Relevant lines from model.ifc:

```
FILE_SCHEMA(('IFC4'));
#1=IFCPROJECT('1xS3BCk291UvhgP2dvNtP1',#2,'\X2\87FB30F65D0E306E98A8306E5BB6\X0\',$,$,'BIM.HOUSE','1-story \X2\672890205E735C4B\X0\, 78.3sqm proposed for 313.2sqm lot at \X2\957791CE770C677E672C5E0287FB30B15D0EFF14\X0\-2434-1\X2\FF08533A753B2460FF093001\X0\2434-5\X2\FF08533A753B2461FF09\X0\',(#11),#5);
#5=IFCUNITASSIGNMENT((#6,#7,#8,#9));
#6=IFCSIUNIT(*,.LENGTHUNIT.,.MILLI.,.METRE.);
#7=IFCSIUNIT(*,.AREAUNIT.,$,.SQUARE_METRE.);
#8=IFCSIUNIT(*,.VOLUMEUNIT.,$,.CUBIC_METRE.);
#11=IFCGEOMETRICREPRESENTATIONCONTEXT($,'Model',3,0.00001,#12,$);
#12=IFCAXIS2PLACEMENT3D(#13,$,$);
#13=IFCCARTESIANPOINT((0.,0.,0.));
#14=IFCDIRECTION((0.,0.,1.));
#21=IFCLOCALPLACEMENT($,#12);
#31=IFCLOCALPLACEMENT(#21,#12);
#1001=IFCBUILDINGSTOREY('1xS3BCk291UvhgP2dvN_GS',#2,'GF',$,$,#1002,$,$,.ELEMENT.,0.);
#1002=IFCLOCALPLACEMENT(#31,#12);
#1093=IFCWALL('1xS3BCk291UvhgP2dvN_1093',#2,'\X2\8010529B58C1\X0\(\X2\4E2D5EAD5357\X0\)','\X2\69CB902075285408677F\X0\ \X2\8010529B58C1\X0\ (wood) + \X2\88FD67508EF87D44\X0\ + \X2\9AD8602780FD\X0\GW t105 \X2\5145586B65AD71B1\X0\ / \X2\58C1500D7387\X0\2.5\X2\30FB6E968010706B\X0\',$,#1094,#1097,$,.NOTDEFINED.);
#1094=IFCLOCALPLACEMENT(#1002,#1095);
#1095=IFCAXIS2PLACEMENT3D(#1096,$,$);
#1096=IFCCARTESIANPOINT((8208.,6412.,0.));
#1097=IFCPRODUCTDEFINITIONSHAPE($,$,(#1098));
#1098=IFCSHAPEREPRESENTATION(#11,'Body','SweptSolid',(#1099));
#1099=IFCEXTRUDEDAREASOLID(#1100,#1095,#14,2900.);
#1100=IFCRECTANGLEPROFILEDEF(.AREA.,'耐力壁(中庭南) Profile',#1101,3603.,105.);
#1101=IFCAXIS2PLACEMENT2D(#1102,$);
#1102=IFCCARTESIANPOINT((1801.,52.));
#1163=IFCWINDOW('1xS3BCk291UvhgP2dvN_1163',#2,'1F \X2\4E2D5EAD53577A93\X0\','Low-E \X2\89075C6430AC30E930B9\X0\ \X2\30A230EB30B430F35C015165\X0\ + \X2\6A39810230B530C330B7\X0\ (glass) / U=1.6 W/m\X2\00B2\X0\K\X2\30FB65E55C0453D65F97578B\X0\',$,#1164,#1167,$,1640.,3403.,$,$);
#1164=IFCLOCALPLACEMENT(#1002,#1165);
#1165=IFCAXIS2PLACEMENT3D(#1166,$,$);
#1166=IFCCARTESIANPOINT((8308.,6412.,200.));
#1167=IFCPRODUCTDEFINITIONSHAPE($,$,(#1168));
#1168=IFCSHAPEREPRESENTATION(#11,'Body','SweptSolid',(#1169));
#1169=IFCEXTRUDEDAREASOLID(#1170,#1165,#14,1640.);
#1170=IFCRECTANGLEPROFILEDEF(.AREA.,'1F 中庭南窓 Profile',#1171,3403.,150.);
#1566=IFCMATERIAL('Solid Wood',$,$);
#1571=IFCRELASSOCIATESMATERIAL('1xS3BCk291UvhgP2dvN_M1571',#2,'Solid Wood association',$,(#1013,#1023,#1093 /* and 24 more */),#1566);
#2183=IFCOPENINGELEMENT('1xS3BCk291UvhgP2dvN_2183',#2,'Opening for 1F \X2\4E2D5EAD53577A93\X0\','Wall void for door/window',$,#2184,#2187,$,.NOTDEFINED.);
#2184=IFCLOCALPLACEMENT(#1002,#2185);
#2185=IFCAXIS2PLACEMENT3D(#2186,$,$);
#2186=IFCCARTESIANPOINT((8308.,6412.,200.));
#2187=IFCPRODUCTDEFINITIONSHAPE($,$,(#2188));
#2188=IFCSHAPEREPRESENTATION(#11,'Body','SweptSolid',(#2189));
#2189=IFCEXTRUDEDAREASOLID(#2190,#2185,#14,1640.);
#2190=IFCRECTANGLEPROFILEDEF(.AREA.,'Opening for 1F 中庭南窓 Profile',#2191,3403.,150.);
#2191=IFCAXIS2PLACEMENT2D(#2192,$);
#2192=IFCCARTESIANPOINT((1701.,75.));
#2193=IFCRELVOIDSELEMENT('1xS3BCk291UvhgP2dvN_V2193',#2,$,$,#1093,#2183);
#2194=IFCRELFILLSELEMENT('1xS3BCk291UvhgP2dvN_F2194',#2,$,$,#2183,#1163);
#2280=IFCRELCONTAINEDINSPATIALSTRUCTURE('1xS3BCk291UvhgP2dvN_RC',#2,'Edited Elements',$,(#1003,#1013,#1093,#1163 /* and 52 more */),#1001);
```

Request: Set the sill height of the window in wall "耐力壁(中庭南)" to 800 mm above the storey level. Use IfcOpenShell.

```python
import numpy as np
import ifcopenshell
import ifcopenshell.api.geometry
import ifcopenshell.geom
import ifcopenshell.util.element
import ifcopenshell.util.placement
import ifcopenshell.util.shape
import ifcopenshell.util.unit

model = ifcopenshell.open("model.ifc")
unit_scale = ifcopenshell.util.unit.calculate_unit_scale(model)

window = model.by_id(1163)
opening = window.FillsVoids[0].RelatingOpeningElement
storey = ifcopenshell.util.element.get_container(window, ifc_class="IfcBuildingStorey")
level = ifcopenshell.util.placement.get_local_placement(storey.ObjectPlacement)[2, 3]

# The opening's origin need not be at the sill, so measure its lowest point.
shape = ifcopenshell.geom.create_shape(ifcopenshell.geom.settings(), opening)
bottom = ifcopenshell.util.shape.get_shape_bottom_elevation(shape, shape.geometry) / unit_scale
dz = level + 0.8 / unit_scale - bottom

shift = np.array([0.0, 0.0, dz])
# The window is not placed relative to its opening, so move both.
for product in (opening, window):
    matrix = ifcopenshell.util.placement.get_local_placement(product.ObjectPlacement)
    matrix[:3, 3] += shift
    ifcopenshell.api.geometry.edit_object_placement(model, product=product, matrix=matrix, is_si=False)

print(f"moved by {dz * unit_scale:+.3f} m")

model.write("model-out.ifc")
```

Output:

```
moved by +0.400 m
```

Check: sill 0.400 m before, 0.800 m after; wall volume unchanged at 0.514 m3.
